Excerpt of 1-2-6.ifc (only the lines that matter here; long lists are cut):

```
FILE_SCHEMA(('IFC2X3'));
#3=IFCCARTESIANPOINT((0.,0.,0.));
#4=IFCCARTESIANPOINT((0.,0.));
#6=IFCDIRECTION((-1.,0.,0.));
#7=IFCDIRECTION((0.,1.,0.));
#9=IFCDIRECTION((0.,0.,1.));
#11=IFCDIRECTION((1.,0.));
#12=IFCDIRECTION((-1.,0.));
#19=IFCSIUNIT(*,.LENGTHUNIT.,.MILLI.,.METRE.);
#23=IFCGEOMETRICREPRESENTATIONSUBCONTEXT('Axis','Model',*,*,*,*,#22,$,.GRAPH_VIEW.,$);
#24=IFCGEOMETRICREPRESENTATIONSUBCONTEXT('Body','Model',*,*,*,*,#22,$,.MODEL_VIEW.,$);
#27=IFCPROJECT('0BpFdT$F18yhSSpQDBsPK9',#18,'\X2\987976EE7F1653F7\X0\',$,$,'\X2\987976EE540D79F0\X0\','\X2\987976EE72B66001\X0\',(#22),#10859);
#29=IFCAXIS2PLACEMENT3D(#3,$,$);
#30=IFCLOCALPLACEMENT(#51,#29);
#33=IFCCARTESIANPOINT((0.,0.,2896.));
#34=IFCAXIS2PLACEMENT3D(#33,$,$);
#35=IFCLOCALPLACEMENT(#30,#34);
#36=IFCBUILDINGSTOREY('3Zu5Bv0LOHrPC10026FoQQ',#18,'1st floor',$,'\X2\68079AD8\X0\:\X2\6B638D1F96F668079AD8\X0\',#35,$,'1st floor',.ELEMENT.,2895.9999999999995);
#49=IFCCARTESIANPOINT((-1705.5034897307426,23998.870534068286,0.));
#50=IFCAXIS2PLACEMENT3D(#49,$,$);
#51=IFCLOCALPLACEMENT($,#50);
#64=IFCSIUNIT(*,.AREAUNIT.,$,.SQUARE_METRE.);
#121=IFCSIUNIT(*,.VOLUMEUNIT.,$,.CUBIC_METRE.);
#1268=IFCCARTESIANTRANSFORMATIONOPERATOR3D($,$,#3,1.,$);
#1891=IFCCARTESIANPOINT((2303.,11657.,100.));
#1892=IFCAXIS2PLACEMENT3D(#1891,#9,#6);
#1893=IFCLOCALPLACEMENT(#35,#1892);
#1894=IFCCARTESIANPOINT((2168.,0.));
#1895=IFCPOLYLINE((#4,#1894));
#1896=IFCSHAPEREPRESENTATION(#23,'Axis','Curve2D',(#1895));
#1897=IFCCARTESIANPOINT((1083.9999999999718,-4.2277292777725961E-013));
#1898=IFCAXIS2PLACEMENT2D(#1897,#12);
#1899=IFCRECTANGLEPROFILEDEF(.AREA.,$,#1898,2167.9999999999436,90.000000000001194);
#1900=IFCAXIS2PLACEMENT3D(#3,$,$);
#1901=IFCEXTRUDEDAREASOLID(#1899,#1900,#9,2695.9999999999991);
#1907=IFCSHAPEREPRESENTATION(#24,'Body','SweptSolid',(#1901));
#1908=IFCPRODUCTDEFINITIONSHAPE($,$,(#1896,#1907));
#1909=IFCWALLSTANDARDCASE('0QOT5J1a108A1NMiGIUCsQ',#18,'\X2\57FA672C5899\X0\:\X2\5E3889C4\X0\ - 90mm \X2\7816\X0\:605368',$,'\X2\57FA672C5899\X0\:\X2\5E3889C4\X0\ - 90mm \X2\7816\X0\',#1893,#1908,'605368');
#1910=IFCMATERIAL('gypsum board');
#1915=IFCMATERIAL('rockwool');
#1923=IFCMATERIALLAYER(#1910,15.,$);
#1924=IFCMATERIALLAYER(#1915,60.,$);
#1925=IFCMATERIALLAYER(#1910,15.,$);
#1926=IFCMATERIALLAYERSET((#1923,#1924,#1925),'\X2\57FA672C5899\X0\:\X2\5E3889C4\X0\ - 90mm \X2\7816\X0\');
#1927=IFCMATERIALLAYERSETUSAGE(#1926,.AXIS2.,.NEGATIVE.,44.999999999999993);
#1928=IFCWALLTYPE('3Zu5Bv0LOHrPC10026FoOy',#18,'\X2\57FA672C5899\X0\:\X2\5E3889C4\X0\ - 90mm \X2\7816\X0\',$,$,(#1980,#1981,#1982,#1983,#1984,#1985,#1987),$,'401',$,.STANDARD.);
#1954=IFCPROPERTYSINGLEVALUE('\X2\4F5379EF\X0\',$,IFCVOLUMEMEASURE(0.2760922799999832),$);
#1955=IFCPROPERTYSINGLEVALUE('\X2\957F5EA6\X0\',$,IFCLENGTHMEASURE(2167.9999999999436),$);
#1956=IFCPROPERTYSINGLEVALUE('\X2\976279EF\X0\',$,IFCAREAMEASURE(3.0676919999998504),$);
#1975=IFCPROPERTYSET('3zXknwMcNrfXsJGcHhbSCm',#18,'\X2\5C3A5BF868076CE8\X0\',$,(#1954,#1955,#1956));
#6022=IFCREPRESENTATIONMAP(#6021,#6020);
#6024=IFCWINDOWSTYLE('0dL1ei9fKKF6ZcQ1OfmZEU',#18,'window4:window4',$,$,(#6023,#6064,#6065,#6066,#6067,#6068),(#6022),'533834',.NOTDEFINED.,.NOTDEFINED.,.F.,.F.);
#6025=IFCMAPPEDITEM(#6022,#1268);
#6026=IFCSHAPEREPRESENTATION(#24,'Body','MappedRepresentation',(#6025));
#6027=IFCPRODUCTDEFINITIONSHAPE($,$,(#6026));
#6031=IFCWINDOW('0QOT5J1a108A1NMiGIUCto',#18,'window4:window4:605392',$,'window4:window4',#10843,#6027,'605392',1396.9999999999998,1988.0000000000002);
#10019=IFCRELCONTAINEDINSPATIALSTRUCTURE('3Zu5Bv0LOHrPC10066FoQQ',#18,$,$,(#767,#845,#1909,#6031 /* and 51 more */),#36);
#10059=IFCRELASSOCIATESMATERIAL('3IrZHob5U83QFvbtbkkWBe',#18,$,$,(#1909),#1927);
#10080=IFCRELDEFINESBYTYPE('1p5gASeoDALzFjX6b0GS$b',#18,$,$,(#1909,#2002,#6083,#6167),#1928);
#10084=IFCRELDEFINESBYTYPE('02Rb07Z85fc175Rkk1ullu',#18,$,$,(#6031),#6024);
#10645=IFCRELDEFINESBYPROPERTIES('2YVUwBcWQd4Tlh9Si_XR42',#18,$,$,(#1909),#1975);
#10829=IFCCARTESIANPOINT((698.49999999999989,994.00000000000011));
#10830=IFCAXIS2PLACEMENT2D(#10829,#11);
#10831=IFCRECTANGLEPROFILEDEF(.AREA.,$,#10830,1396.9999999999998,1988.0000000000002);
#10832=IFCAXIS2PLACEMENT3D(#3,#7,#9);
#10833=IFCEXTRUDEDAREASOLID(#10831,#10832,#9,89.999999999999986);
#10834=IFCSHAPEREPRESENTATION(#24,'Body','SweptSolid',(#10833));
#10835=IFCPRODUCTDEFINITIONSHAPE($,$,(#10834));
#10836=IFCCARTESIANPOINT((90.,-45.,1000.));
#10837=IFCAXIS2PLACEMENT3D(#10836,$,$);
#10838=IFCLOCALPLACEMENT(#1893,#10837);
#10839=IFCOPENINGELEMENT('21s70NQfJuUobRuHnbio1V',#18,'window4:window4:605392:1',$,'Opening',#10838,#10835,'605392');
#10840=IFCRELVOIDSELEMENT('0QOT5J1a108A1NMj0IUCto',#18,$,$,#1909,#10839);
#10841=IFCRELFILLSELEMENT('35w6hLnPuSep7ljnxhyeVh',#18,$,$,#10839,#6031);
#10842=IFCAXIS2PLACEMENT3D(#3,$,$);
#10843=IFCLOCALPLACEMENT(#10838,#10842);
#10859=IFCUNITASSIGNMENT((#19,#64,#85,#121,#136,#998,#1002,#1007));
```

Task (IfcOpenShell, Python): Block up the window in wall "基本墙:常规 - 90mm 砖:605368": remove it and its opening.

```python
import ifcopenshell
import ifcopenshell.api.feature
import ifcopenshell.api.pset
import ifcopenshell.api.root
import ifcopenshell.geom
import ifcopenshell.util.element
import ifcopenshell.util.shape
import ifcopenshell.util.unit

model = ifcopenshell.open("1-2-6.ifc")
area_scale = ifcopenshell.util.unit.calculate_unit_scale(model, "AREAUNIT")
volume_scale = ifcopenshell.util.unit.calculate_unit_scale(model, "VOLUMEUNIT")
settings = ifcopenshell.geom.settings()


def volume(element):
    """Net volume in cubic metres, openings subtracted."""
    shape = ifcopenshell.geom.create_shape(settings, element)
    return ifcopenshell.util.shape.get_volume(shape.geometry)


window = model.by_guid("0QOT5J1a108A1NMiGIUCto")
opening = window.FillsVoids[0].RelatingOpeningElement
wall = opening.VoidsElements[0].RelatingBuildingElement
before = volume(wall)

ifcopenshell.api.root.remove_product(model, product=window)
ifcopenshell.api.feature.remove_feature(model, feature=opening)

after = volume(wall)
thickness = 0.09  # wall thickness in metres

# Update the wall's stored quantities.
pset = model.by_id(ifcopenshell.util.element.get_pset(wall, "尺寸标注", should_inherit=False)["id"])
ifcopenshell.api.pset.edit_pset(model, pset=pset, properties={
    "体积": model.create_entity("IfcVolumeMeasure", after / volume_scale),
    "面积": model.create_entity("IfcAreaMeasure", after / thickness / area_scale),
})

print(f"wall volume {before:.3f} -> {after:.3f} m3")

model.write("1-2-6_edited.ifc")
```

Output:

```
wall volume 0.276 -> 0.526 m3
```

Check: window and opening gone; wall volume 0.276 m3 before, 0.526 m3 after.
